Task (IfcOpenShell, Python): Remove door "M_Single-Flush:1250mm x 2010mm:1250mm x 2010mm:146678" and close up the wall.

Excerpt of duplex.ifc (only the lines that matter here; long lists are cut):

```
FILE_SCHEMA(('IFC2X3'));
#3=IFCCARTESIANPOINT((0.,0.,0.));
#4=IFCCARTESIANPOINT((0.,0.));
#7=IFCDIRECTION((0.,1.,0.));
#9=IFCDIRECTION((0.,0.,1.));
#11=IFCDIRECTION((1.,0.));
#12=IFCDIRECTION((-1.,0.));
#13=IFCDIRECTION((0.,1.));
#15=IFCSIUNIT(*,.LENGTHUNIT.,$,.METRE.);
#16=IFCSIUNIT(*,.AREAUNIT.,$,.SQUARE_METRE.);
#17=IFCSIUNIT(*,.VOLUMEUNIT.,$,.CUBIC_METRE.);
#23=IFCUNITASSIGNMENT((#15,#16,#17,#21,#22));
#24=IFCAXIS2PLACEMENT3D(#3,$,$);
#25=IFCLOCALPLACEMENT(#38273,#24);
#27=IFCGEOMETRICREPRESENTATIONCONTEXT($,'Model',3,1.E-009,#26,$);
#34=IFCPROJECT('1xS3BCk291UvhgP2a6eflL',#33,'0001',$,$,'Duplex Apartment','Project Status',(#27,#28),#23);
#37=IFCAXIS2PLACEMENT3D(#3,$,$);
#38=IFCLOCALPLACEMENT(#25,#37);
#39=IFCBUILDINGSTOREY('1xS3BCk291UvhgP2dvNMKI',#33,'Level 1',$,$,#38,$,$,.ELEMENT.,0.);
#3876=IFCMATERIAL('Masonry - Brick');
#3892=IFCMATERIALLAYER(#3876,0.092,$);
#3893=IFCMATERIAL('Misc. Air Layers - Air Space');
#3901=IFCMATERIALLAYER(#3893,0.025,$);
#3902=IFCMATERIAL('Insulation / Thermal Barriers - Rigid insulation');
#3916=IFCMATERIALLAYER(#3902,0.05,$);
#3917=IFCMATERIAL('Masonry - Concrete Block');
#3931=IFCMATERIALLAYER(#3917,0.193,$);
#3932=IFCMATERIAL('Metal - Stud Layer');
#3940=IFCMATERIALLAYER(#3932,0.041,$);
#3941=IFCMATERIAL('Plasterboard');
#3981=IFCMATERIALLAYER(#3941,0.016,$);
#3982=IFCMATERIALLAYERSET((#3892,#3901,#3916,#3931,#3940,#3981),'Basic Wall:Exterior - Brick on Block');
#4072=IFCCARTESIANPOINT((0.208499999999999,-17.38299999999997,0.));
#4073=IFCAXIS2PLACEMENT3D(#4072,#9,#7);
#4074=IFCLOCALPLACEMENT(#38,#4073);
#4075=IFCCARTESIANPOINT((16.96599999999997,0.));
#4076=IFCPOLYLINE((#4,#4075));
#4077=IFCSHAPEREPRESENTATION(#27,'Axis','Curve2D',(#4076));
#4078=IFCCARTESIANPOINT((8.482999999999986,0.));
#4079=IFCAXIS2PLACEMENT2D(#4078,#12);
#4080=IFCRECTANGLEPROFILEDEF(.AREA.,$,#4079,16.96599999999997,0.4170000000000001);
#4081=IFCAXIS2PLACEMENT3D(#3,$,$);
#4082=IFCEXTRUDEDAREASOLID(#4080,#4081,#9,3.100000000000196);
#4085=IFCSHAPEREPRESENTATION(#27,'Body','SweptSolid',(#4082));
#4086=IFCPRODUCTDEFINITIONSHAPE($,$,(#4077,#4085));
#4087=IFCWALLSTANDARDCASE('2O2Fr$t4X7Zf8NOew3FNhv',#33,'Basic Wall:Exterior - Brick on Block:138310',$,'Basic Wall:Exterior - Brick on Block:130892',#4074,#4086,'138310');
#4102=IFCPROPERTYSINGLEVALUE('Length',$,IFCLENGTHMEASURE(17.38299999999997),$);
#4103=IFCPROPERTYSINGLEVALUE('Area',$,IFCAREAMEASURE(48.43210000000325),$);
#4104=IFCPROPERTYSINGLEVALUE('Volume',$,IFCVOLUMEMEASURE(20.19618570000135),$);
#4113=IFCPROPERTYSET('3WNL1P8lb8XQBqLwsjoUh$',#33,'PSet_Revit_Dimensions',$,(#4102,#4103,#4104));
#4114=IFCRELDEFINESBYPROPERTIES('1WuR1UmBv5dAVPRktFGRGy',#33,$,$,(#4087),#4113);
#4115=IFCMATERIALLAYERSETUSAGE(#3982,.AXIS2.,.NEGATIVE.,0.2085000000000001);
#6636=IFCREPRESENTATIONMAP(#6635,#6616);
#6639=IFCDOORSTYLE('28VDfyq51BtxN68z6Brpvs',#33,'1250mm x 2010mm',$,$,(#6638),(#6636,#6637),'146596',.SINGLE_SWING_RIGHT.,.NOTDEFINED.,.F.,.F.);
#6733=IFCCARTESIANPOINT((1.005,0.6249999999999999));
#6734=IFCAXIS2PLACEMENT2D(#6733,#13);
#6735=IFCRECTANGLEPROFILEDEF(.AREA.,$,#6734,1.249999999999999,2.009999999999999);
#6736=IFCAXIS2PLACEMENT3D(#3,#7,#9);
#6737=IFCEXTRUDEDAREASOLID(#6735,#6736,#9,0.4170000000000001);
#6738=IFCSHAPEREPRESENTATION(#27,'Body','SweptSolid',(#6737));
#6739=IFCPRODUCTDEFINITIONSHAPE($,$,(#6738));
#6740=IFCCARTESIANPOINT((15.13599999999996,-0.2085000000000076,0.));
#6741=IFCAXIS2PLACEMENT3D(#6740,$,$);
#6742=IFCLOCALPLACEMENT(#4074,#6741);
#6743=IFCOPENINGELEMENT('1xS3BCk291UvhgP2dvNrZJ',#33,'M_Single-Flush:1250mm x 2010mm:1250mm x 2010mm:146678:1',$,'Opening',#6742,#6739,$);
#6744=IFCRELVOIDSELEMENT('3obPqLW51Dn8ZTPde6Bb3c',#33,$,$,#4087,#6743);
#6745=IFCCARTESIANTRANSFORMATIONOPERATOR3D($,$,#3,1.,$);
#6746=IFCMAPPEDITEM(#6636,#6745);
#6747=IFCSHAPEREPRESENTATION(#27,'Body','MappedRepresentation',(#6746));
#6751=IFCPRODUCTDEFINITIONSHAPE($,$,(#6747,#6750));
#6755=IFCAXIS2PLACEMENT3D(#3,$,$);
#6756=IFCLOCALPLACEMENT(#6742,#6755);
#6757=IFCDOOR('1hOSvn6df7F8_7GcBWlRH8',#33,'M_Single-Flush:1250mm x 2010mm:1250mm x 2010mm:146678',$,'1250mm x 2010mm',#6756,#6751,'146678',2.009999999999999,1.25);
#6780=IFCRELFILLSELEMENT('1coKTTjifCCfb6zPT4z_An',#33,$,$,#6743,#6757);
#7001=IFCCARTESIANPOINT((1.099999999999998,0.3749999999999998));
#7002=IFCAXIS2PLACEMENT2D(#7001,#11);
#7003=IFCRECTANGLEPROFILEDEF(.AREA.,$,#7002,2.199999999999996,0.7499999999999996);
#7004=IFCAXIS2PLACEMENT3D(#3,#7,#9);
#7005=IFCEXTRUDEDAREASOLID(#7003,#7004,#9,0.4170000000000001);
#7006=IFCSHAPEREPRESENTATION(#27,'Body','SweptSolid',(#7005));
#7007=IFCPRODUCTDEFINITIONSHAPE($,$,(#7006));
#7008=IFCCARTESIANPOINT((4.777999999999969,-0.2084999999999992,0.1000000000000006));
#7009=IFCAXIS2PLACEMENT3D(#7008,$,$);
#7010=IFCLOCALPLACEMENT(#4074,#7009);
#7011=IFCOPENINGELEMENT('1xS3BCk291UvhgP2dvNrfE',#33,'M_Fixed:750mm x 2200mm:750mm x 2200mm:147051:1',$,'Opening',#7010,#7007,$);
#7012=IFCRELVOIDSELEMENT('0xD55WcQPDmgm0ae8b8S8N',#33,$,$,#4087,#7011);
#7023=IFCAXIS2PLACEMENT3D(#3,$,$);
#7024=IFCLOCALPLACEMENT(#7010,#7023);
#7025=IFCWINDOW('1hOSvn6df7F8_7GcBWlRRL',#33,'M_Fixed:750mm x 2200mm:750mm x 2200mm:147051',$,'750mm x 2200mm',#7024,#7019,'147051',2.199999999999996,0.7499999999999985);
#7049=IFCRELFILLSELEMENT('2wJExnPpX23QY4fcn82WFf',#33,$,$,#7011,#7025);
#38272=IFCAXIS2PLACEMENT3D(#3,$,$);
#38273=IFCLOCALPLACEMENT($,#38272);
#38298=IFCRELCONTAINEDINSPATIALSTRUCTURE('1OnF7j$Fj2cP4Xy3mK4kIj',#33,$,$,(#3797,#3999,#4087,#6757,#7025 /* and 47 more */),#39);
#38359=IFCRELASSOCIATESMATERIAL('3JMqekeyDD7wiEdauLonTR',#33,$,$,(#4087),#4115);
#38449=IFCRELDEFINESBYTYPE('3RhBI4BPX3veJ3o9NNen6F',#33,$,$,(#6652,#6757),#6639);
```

```python
import ifcopenshell
import ifcopenshell.api.feature
import ifcopenshell.api.pset
import ifcopenshell.api.root
import ifcopenshell.geom
import ifcopenshell.util.element
import ifcopenshell.util.shape
import ifcopenshell.util.unit

model = ifcopenshell.open("duplex.ifc")
area_scale = ifcopenshell.util.unit.calculate_unit_scale(model, "AREAUNIT")
volume_scale = ifcopenshell.util.unit.calculate_unit_scale(model, "VOLUMEUNIT")
settings = ifcopenshell.geom.settings()


def volume(element):
    """Net volume in cubic metres, openings subtracted."""
    shape = ifcopenshell.geom.create_shape(settings, element)
    return ifcopenshell.util.shape.get_volume(shape.geometry)


door = model.by_guid("1hOSvn6df7F8_7GcBWlRH8")
opening = door.FillsVoids[0].RelatingOpeningElement
wall = opening.VoidsElements[0].RelatingBuildingElement
before = volume(wall)

ifcopenshell.api.root.remove_product(model, product=door)
ifcopenshell.api.feature.remove_feature(model, feature=opening)

after = volume(wall)
thickness = 0.417  # wall thickness in metres

# Update the wall's stored quantities.
pset = model.by_id(ifcopenshell.util.element.get_pset(wall, "PSet_Revit_Dimensions", should_inherit=False)["id"])
ifcopenshell.api.pset.edit_pset(model, pset=pset, properties={
    "Area": model.create_entity("IfcAreaMeasure", after / thickness / area_scale),
    "Volume": model.create_entity("IfcVolumeMeasure", after / volume_scale),
})

print(f"wall volume {before:.3f} -> {after:.3f} m3")

model.write("duplex_updated.ifc")
```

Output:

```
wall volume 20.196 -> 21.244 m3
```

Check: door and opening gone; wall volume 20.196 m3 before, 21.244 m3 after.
